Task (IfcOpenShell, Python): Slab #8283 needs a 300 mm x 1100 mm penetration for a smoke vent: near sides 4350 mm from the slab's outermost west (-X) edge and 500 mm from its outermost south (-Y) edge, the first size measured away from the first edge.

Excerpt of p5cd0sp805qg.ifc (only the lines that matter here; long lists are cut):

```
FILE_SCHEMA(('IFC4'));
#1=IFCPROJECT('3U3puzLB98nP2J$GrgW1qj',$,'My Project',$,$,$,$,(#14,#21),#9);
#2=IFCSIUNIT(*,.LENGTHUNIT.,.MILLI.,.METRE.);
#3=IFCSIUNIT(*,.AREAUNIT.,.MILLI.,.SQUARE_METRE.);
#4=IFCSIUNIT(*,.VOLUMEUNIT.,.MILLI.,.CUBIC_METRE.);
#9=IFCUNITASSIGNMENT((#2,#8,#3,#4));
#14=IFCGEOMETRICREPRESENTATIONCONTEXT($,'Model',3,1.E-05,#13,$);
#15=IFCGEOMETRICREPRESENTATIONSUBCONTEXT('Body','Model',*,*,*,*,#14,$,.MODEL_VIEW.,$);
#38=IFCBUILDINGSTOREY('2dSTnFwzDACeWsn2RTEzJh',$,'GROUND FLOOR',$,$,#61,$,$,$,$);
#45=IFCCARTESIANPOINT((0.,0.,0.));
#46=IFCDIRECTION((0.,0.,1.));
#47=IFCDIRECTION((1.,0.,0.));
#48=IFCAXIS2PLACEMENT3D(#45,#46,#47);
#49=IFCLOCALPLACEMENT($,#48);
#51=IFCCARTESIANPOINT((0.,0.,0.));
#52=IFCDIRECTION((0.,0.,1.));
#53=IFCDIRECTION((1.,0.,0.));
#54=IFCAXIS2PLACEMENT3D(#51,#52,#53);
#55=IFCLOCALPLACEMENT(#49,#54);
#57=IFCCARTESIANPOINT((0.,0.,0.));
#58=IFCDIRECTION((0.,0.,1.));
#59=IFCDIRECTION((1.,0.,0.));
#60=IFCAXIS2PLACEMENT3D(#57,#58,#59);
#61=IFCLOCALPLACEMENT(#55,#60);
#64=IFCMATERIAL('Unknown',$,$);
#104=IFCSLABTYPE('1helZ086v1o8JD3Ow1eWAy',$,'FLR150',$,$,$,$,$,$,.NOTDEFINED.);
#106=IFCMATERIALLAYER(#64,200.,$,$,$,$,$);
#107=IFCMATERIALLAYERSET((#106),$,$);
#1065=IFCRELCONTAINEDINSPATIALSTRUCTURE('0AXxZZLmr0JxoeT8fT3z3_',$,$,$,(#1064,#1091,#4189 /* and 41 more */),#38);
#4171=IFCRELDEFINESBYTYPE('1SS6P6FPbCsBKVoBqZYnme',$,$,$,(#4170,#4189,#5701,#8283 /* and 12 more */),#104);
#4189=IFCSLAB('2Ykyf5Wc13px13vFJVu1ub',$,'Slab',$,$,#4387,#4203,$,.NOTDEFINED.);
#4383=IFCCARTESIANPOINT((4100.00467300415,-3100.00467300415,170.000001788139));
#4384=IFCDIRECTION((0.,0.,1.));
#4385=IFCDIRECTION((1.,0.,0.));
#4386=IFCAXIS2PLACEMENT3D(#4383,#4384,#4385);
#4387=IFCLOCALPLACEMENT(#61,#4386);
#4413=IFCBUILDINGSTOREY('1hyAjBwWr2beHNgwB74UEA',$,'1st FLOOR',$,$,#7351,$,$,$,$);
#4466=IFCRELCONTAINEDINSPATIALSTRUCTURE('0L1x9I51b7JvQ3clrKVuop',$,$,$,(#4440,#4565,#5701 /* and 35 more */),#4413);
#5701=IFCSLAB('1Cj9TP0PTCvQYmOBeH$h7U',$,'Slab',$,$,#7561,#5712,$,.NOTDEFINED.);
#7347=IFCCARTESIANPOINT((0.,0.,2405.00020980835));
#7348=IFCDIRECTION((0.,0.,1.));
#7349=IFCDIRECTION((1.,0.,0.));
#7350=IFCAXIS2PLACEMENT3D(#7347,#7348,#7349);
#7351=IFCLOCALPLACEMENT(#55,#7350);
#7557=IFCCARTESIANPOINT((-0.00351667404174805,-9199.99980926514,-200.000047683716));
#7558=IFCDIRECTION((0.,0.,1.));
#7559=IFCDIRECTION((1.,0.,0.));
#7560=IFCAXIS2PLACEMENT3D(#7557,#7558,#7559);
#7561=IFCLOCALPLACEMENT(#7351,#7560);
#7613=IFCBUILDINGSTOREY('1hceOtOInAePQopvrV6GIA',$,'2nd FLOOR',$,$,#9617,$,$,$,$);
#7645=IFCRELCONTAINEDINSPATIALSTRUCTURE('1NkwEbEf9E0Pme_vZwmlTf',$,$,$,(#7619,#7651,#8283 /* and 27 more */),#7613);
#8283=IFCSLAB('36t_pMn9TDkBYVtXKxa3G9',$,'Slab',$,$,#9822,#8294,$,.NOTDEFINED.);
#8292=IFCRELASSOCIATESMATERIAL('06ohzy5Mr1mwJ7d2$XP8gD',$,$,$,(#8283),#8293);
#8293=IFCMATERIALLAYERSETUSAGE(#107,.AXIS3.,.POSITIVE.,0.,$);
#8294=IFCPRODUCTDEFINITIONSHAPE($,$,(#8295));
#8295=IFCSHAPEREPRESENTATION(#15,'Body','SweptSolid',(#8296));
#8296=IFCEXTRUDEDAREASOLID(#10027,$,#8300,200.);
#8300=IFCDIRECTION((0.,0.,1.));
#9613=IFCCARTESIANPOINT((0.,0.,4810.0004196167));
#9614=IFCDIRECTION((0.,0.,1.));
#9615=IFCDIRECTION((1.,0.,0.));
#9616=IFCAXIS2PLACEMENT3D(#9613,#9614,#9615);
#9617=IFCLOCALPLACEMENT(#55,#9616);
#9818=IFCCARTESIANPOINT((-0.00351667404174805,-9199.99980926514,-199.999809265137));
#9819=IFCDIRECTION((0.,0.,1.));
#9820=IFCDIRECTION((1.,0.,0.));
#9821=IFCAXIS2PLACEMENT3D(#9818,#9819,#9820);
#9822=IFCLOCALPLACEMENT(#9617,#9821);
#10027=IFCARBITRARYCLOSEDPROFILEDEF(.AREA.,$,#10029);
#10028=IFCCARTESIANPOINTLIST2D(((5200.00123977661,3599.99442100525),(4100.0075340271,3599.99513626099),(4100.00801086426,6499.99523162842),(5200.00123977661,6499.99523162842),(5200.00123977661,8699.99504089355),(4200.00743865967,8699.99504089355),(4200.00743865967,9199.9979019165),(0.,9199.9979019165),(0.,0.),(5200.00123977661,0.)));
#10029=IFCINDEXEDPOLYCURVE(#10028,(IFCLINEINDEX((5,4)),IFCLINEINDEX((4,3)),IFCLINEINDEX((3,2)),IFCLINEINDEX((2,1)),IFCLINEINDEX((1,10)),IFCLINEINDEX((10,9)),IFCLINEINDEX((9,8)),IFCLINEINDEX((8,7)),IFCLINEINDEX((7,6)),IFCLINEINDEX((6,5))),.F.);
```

```python
import numpy as np
import ifcopenshell
import ifcopenshell.api.feature
import ifcopenshell.api.geometry
import ifcopenshell.api.root
import ifcopenshell.geom
import ifcopenshell.util.placement
import ifcopenshell.util.representation
import ifcopenshell.util.shape
import ifcopenshell.util.unit

model = ifcopenshell.open("p5cd0sp805qg.ifc")
unit_scale = ifcopenshell.util.unit.calculate_unit_scale(model)
settings = ifcopenshell.geom.settings()


def volume(element):
    """Net volume in cubic metres, openings subtracted."""
    shape = ifcopenshell.geom.create_shape(settings, element)
    return ifcopenshell.util.shape.get_volume(shape.geometry)


slab = model.by_guid("36t_pMn9TDkBYVtXKxa3G9")
before = volume(slab)

# Extent in the slab's own axes, in metres. The edges named are its -X and -Y sides.
slab_shape = ifcopenshell.geom.create_shape(settings, slab)
vertices = ifcopenshell.util.shape.get_vertices(slab_shape.geometry)
x_min, y_min, bottom = vertices.min(axis=0)
top = vertices[:, 2].max()

opening = ifcopenshell.api.root.create_entity(model, ifc_class="IfcOpeningElement", name="Smoke vent opening", predefined_type="OPENING")
context = ifcopenshell.util.representation.get_context(model, "Model", "Body", "MODEL_VIEW")
width, depth = 0.3, 1.1
outline = [(0.0, 0.0), (width, 0.0), (width, depth), (0.0, depth), (0.0, 0.0)]
# Overshoot both faces by 50 mm so the cut is clean.
shape = ifcopenshell.api.geometry.add_slab_representation(
    model, context=context, depth=top - bottom + 0.1, polyline=outline
)
ifcopenshell.api.geometry.assign_representation(model, product=opening, representation=shape)

matrix = ifcopenshell.util.placement.get_local_placement(slab.ObjectPlacement)
matrix[:, 3] = matrix @ np.append(np.array([x_min + 4.35, y_min + 0.5, bottom - 0.05]) / unit_scale, 1.0)
ifcopenshell.api.geometry.edit_object_placement(model, product=opening, matrix=matrix, is_si=False)
ifcopenshell.api.feature.add_feature(model, feature=opening, element=slab)

after = volume(slab)

print(f"slab volume {before:.3f} -> {after:.3f} m3")

model.write("p5cd0sp805qg_v2.ifc")
```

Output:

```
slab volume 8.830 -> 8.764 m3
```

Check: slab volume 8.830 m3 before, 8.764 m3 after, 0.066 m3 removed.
